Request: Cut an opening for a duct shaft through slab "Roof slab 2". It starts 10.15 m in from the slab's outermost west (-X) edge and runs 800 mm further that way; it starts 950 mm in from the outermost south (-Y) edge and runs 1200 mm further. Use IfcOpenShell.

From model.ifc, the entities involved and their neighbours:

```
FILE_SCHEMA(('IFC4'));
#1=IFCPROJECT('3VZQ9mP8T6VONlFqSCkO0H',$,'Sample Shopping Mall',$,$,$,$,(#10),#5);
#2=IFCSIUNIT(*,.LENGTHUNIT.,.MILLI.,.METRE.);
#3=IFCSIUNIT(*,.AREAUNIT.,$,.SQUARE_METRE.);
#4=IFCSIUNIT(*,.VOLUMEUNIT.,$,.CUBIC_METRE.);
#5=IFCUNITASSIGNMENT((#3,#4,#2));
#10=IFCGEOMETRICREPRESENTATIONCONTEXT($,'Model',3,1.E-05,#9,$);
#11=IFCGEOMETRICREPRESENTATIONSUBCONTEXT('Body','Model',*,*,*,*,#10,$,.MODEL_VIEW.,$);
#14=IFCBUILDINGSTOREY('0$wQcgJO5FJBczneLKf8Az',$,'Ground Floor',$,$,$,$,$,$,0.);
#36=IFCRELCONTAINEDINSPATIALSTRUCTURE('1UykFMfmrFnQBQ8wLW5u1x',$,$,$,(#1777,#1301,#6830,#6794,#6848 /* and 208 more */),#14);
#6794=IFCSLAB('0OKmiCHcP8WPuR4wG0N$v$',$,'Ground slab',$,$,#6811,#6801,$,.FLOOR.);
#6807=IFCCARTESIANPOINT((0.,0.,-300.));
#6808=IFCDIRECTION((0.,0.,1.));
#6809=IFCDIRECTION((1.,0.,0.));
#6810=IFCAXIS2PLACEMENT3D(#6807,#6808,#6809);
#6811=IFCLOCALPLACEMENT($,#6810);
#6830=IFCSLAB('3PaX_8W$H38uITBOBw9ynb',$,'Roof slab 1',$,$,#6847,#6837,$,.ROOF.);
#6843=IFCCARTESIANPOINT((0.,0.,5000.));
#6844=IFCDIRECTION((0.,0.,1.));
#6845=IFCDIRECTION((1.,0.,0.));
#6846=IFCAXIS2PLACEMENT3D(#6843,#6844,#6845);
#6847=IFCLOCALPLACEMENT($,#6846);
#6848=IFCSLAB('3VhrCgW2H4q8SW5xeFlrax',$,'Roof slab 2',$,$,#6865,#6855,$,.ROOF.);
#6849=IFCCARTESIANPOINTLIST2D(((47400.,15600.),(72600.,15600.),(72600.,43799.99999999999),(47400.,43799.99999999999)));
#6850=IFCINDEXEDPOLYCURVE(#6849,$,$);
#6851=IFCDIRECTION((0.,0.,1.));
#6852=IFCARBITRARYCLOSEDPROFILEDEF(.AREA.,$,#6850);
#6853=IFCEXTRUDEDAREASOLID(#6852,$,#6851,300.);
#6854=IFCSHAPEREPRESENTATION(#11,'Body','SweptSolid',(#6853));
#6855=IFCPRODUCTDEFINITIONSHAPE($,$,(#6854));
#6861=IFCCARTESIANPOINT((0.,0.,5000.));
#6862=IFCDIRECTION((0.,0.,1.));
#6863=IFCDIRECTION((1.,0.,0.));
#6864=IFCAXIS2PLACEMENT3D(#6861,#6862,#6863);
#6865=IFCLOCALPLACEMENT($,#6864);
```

```python
import numpy as np
import ifcopenshell
import ifcopenshell.api.feature
import ifcopenshell.api.geometry
import ifcopenshell.api.root
import ifcopenshell.geom
import ifcopenshell.util.placement
import ifcopenshell.util.representation
import ifcopenshell.util.shape
import ifcopenshell.util.unit

model = ifcopenshell.open("model.ifc")
unit_scale = ifcopenshell.util.unit.calculate_unit_scale(model)
settings = ifcopenshell.geom.settings()


def volume(element):
    """Net volume in cubic metres, openings subtracted."""
    shape = ifcopenshell.geom.create_shape(settings, element)
    return ifcopenshell.util.shape.get_volume(shape.geometry)


slab = model.by_guid("3VhrCgW2H4q8SW5xeFlrax")
before = volume(slab)

# Extent in the slab's own axes, in metres. The edges named are its -X and -Y sides.
slab_shape = ifcopenshell.geom.create_shape(settings, slab)
vertices = ifcopenshell.util.shape.get_vertices(slab_shape.geometry)
x_min, y_min, bottom = vertices.min(axis=0)
top = vertices[:, 2].max()

opening = ifcopenshell.api.root.create_entity(model, ifc_class="IfcOpeningElement", name="Duct shaft opening", predefined_type="OPENING")
context = ifcopenshell.util.representation.get_context(model, "Model", "Body", "MODEL_VIEW")
width, depth = 0.8, 1.2
outline = [(0.0, 0.0), (width, 0.0), (width, depth), (0.0, depth), (0.0, 0.0)]
# Overshoot both faces by 50 mm so the cut is clean.
shape = ifcopenshell.api.geometry.add_slab_representation(
    model, context=context, depth=top - bottom + 0.1, polyline=outline
)
ifcopenshell.api.geometry.assign_representation(model, product=opening, representation=shape)

matrix = ifcopenshell.util.placement.get_local_placement(slab.ObjectPlacement)
matrix[:, 3] = matrix @ np.append(np.array([x_min + 10.15, y_min + 0.95, bottom - 0.05]) / unit_scale, 1.0)
ifcopenshell.api.geometry.edit_object_placement(model, product=opening, matrix=matrix, is_si=False)
ifcopenshell.api.feature.add_feature(model, feature=opening, element=slab)

after = volume(slab)

print(f"slab volume {before:.3f} -> {after:.3f} m3")

model.write("model-out.ifc")
```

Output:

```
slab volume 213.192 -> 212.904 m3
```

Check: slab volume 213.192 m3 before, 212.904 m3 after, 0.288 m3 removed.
